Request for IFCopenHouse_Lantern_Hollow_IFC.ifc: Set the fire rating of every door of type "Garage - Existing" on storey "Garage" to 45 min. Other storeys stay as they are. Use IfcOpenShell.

First a look at what the model holds.

```python
import ifcopenshell
import ifcopenshell.util.element

model = ifcopenshell.open("IFCopenHouse_Lantern_Hollow_IFC.ifc")
print(model.schema)
storey = next(s for s in model.by_type("IfcBuildingStorey") if s.Name == "Garage")
doors = [e for e in ifcopenshell.util.element.get_decomposition(storey) if e.is_a("IfcDoor")]
seen = {}
for e in doors:
    element_type = ifcopenshell.util.element.get_type(e)
    key = (element_type.Name if element_type != e and element_type else None, ifcopenshell.util.element.get_pset(e, "Pset_DoorCommon", "FireRating"))
    seen[key] = seen.get(key, 0) + 1
for (name, value), count in sorted(seen.items(), key=str):
    print(count, "x", name, "|", value)
```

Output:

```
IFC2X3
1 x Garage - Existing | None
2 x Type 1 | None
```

```python
import ifcopenshell
import ifcopenshell.api.pset
import ifcopenshell.util.element

model = ifcopenshell.open("IFCopenHouse_Lantern_Hollow_IFC.ifc")

storey = next(s for s in model.by_type("IfcBuildingStorey") if s.Name == "Garage")
doors = [e for e in ifcopenshell.util.element.get_decomposition(storey) if e.is_a("IfcDoor")]

count = 0
for e in doors:
    element_type = ifcopenshell.util.element.get_type(e)
    if element_type in (None, e) or element_type.Name != "Garage - Existing":
        continue
    # add_pset returns the element's existing set when there is one.
    pset = ifcopenshell.api.pset.add_pset(model, product=e, name="Pset_DoorCommon")
    ifcopenshell.api.pset.edit_pset(model, pset=pset, properties={"FireRating": "45 min"})
    count += 1

print(count, "doors updated")

model.write("IFCopenHouse_Lantern_Hollow_IFC_updated.ifc")
```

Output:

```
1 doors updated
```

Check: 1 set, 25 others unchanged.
